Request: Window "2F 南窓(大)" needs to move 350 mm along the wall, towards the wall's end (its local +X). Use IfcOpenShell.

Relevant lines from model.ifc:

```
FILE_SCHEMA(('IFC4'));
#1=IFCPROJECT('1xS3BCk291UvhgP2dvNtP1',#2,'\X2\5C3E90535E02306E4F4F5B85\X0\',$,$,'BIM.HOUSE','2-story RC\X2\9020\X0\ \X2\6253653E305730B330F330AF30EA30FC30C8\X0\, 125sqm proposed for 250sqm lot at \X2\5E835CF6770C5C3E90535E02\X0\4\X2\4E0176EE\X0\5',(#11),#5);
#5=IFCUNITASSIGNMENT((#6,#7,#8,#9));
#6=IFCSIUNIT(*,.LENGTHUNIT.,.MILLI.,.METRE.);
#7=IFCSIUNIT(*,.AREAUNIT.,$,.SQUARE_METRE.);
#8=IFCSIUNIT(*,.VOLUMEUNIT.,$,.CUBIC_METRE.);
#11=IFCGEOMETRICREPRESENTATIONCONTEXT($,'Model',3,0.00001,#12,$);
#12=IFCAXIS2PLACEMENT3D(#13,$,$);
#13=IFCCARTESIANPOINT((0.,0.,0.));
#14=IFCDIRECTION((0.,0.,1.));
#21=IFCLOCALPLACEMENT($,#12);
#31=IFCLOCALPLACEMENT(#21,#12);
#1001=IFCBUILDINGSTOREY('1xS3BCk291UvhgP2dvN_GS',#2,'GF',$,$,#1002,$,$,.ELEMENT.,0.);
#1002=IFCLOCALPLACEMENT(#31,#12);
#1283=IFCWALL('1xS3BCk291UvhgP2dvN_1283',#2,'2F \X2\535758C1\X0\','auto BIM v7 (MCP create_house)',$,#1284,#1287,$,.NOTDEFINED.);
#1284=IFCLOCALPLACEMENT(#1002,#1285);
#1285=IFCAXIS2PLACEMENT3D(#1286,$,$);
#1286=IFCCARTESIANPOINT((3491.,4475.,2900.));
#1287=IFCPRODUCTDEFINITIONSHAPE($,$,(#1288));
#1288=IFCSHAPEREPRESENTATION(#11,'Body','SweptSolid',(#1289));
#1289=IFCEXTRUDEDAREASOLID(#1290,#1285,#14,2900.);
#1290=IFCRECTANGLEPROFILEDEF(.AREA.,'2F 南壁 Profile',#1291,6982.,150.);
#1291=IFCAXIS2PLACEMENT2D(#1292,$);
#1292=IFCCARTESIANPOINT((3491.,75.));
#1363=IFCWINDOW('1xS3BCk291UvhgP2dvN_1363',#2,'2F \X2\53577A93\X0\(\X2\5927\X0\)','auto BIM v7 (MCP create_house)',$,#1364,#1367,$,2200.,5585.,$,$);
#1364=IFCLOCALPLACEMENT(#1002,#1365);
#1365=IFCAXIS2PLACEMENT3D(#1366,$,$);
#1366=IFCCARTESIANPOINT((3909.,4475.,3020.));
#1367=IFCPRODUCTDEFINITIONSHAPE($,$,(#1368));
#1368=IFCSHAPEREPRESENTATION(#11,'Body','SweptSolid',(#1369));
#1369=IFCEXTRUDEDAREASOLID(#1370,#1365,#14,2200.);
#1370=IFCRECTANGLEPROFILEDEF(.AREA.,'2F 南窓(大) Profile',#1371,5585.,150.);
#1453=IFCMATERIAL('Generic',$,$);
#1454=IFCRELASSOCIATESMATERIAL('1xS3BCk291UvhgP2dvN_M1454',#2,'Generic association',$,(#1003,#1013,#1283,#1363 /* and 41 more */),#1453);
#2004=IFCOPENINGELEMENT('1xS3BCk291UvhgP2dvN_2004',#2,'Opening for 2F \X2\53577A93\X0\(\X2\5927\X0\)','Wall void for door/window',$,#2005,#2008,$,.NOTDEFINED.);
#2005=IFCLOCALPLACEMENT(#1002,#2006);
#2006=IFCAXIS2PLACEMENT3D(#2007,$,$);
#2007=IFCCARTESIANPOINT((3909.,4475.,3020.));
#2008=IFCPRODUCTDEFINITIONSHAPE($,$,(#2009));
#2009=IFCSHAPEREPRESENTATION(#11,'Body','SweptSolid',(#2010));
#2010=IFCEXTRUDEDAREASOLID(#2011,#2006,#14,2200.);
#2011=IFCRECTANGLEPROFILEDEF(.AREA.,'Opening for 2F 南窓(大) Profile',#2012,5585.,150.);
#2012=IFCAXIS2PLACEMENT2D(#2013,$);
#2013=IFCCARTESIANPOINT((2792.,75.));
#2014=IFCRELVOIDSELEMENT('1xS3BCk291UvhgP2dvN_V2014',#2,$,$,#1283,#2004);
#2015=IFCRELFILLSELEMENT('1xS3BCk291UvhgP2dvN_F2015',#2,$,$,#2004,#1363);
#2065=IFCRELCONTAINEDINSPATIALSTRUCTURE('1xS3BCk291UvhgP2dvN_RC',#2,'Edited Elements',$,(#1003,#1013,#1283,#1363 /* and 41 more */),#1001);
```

```python
import ifcopenshell
import ifcopenshell.api.geometry
import ifcopenshell.util.placement
import ifcopenshell.util.unit

model = ifcopenshell.open("model.ifc")
unit_scale = ifcopenshell.util.unit.calculate_unit_scale(model)

window = model.by_id(1363)
opening = window.FillsVoids[0].RelatingOpeningElement
wall = opening.VoidsElements[0].RelatingBuildingElement

wall_matrix = ifcopenshell.util.placement.get_local_placement(wall.ObjectPlacement)
shift = wall_matrix[:3, 0] * 0.35 / unit_scale
before = ifcopenshell.util.placement.get_local_placement(window.ObjectPlacement)[:3, 3].copy()

# The window is not placed relative to its opening, so move both.
for product in (opening, window):
    matrix = ifcopenshell.util.placement.get_local_placement(product.ObjectPlacement)
    matrix[:3, 3] += shift
    ifcopenshell.api.geometry.edit_object_placement(model, product=product, matrix=matrix, is_si=False)

after = ifcopenshell.util.placement.get_local_placement(window.ObjectPlacement)[:3, 3]
print("window moved by", (after - before).round(3) + 0.0)

model.write("model_updated.ifc")
```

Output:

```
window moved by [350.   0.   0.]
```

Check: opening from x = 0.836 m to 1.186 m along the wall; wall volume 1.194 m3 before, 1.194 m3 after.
